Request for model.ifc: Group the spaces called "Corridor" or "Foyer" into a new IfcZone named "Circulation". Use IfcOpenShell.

First a look at what the model holds.

```python
import ifcopenshell

model = ifcopenshell.open("model.ifc")
print(model.schema)
seen = {}
for space in model.by_type("IfcSpace"):
    seen[space.LongName] = seen.get(space.LongName, 0) + 1
for name, count in sorted(seen.items(), key=str):
    print(count, "x", name)
print("zones:", [z.Name for z in model.by_type("IfcZone")][:20])
```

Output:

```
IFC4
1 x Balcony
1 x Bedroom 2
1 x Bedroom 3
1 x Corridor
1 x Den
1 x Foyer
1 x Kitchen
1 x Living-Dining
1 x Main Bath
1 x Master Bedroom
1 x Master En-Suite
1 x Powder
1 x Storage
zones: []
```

```python
import ifcopenshell
import ifcopenshell.api.group
import ifcopenshell.api.root

model = ifcopenshell.open("model.ifc")

names = {"Corridor", "Foyer"}
spaces = [s for s in model.by_type("IfcSpace") if s.LongName in names]

zone = ifcopenshell.api.root.create_entity(model, ifc_class="IfcZone", name="Circulation")
ifcopenshell.api.group.assign_group(model, products=spaces, group=zone)
print(len(spaces), "spaces in", zone.Name)

model.write("model-out.ifc")
```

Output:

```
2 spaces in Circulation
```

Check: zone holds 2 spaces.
